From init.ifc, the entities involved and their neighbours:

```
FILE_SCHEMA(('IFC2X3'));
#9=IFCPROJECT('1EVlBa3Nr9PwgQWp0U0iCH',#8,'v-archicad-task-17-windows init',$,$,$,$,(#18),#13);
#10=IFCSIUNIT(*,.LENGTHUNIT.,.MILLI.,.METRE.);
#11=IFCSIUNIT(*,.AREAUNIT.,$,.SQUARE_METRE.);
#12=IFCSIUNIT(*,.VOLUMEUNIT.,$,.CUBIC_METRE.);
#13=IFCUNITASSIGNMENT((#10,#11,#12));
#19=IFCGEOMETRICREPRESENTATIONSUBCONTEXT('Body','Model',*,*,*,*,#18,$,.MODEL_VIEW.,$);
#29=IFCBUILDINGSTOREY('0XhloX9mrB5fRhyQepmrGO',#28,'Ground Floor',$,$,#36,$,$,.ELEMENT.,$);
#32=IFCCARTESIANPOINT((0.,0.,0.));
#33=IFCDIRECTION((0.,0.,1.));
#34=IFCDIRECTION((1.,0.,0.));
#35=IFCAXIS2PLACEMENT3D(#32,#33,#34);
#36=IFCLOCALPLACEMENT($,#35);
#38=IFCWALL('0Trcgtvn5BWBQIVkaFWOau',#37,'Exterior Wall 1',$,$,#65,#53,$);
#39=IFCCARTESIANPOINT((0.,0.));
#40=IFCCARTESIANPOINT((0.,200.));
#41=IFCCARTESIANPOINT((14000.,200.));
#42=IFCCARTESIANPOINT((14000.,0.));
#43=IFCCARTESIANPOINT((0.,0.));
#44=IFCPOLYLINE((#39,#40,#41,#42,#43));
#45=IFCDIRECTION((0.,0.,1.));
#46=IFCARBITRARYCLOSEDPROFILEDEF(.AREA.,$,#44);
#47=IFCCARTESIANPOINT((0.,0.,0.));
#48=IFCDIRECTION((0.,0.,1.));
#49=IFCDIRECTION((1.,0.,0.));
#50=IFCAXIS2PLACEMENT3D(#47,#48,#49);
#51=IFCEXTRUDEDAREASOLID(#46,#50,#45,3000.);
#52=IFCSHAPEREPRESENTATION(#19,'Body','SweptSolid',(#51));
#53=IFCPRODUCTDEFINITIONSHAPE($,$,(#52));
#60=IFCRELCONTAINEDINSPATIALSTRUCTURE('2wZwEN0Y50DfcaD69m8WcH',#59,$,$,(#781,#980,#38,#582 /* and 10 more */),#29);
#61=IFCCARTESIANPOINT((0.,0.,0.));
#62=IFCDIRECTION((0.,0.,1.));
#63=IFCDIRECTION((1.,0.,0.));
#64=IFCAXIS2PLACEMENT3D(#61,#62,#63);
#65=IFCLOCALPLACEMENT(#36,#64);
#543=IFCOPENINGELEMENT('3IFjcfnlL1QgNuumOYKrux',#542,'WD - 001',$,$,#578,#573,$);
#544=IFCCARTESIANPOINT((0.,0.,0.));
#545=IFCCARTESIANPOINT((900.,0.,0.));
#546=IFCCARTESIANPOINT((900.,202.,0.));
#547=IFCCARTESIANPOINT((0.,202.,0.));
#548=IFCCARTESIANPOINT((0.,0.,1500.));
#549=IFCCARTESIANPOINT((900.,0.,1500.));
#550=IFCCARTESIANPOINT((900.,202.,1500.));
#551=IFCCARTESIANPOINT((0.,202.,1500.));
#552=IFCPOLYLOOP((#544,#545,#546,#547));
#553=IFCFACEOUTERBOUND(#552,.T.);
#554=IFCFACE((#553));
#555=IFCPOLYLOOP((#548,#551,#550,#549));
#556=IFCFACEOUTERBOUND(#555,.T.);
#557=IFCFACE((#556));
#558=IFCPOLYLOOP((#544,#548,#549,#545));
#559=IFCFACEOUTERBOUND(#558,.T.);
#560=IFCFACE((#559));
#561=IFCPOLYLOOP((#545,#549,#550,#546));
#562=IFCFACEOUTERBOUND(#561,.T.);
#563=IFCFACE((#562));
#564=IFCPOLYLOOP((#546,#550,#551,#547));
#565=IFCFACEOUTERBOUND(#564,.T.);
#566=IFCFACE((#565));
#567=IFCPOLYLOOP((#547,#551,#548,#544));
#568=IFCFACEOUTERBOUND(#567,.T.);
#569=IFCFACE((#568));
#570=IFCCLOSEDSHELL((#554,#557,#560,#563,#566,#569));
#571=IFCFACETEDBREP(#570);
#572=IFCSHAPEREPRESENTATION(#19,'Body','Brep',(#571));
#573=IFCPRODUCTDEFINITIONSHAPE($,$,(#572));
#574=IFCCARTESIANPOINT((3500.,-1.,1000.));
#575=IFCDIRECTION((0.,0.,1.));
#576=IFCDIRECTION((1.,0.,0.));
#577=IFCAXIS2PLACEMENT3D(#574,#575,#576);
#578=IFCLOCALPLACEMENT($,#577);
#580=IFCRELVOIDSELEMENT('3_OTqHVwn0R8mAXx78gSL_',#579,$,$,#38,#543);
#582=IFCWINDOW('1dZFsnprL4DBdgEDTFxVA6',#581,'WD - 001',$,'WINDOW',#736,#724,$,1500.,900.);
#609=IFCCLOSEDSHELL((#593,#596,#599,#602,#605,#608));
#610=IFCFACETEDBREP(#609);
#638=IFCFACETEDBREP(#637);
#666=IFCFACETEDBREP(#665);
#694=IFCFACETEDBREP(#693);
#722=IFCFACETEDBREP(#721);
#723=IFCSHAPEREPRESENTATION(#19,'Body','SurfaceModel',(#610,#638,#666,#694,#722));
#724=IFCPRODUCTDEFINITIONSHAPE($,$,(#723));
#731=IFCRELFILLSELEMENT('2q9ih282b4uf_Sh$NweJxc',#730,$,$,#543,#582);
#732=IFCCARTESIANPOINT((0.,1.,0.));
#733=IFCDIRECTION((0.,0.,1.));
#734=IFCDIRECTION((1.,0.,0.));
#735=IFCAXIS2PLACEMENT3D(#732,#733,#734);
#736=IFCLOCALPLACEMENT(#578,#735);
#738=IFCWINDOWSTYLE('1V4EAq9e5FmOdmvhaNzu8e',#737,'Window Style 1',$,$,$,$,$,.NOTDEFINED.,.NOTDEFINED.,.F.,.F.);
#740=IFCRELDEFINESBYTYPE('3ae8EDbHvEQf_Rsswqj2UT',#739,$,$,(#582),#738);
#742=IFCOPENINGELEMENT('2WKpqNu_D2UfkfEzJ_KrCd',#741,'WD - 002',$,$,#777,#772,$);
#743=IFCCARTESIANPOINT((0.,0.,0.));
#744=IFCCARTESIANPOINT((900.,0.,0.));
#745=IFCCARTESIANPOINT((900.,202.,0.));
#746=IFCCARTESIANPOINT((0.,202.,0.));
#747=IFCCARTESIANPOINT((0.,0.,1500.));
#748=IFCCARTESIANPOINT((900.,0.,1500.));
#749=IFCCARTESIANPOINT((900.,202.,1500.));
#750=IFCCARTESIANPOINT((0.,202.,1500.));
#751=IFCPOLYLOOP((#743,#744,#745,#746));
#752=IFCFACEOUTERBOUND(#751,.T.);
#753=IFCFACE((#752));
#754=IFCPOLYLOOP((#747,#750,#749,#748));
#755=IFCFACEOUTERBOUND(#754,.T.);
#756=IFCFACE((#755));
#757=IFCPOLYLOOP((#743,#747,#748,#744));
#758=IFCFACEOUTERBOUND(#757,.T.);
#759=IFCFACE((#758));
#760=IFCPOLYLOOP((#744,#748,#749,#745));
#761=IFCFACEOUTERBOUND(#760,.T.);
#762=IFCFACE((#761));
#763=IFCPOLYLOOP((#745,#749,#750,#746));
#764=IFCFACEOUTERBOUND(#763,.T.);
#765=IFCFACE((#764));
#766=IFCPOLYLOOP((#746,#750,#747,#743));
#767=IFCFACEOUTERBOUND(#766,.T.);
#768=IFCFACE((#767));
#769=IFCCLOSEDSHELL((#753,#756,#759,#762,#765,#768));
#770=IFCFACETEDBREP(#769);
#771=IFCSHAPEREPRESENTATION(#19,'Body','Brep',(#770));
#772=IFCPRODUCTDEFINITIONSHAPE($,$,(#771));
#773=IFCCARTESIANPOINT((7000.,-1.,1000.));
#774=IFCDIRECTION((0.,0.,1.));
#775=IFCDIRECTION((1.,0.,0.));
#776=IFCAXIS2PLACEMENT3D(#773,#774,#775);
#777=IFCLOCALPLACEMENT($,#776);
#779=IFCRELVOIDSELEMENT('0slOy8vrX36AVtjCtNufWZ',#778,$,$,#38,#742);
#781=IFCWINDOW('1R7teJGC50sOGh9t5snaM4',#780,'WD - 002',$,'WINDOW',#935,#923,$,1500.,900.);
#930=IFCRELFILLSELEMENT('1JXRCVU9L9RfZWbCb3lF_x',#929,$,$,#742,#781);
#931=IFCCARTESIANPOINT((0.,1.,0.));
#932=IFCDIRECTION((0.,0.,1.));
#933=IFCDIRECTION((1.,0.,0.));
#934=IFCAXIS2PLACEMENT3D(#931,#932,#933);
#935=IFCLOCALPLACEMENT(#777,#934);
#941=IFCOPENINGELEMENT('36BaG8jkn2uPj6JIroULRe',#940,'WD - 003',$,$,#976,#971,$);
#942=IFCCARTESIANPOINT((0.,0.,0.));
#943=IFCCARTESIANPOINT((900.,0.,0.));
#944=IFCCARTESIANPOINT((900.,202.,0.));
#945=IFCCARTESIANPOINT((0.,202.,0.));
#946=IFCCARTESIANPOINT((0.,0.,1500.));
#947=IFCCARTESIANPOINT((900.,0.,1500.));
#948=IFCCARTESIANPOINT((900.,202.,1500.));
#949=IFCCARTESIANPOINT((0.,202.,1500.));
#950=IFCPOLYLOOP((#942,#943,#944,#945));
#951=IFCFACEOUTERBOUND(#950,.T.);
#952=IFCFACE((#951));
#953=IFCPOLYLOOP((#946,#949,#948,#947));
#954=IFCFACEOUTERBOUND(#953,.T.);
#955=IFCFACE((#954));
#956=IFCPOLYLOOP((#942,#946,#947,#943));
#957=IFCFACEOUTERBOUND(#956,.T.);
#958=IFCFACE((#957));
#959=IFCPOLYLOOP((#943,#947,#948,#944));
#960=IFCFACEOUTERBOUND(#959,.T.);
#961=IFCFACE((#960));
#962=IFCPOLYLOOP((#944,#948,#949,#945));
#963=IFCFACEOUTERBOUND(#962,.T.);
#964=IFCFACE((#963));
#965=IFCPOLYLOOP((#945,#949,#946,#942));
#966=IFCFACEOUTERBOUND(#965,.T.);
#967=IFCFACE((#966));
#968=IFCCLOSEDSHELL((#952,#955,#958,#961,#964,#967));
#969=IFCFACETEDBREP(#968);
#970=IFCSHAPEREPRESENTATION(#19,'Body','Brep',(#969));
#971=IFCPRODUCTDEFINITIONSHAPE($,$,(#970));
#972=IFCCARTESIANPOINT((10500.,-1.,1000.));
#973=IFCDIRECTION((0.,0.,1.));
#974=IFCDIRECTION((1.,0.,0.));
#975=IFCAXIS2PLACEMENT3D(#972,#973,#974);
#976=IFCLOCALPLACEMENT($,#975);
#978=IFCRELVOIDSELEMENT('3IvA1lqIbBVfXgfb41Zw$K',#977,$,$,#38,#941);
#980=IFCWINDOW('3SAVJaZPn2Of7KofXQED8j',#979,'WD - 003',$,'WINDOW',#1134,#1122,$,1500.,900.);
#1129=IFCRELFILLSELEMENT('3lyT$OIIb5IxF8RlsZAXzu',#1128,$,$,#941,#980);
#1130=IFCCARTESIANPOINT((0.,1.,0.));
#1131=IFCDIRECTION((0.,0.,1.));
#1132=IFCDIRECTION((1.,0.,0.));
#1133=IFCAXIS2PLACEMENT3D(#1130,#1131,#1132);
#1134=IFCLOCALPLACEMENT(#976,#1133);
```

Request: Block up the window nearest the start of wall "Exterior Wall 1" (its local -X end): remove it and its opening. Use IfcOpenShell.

```python
import ifcopenshell
import ifcopenshell.api.feature
import ifcopenshell.api.root
import ifcopenshell.geom
import ifcopenshell.util.shape

model = ifcopenshell.open("init.ifc")
settings = ifcopenshell.geom.settings()


def volume(element):
    """Net volume in cubic metres, openings subtracted."""
    shape = ifcopenshell.geom.create_shape(settings, element)
    return ifcopenshell.util.shape.get_volume(shape.geometry)


window = model.by_guid("1dZFsnprL4DBdgEDTFxVA6")
opening = window.FillsVoids[0].RelatingOpeningElement
wall = opening.VoidsElements[0].RelatingBuildingElement
before = volume(wall)

ifcopenshell.api.root.remove_product(model, product=window)
ifcopenshell.api.feature.remove_feature(model, feature=opening)

after = volume(wall)

print(f"wall volume {before:.3f} -> {after:.3f} m3")

model.write("init_rev.ifc")
```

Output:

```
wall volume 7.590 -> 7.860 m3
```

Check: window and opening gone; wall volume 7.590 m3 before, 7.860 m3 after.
